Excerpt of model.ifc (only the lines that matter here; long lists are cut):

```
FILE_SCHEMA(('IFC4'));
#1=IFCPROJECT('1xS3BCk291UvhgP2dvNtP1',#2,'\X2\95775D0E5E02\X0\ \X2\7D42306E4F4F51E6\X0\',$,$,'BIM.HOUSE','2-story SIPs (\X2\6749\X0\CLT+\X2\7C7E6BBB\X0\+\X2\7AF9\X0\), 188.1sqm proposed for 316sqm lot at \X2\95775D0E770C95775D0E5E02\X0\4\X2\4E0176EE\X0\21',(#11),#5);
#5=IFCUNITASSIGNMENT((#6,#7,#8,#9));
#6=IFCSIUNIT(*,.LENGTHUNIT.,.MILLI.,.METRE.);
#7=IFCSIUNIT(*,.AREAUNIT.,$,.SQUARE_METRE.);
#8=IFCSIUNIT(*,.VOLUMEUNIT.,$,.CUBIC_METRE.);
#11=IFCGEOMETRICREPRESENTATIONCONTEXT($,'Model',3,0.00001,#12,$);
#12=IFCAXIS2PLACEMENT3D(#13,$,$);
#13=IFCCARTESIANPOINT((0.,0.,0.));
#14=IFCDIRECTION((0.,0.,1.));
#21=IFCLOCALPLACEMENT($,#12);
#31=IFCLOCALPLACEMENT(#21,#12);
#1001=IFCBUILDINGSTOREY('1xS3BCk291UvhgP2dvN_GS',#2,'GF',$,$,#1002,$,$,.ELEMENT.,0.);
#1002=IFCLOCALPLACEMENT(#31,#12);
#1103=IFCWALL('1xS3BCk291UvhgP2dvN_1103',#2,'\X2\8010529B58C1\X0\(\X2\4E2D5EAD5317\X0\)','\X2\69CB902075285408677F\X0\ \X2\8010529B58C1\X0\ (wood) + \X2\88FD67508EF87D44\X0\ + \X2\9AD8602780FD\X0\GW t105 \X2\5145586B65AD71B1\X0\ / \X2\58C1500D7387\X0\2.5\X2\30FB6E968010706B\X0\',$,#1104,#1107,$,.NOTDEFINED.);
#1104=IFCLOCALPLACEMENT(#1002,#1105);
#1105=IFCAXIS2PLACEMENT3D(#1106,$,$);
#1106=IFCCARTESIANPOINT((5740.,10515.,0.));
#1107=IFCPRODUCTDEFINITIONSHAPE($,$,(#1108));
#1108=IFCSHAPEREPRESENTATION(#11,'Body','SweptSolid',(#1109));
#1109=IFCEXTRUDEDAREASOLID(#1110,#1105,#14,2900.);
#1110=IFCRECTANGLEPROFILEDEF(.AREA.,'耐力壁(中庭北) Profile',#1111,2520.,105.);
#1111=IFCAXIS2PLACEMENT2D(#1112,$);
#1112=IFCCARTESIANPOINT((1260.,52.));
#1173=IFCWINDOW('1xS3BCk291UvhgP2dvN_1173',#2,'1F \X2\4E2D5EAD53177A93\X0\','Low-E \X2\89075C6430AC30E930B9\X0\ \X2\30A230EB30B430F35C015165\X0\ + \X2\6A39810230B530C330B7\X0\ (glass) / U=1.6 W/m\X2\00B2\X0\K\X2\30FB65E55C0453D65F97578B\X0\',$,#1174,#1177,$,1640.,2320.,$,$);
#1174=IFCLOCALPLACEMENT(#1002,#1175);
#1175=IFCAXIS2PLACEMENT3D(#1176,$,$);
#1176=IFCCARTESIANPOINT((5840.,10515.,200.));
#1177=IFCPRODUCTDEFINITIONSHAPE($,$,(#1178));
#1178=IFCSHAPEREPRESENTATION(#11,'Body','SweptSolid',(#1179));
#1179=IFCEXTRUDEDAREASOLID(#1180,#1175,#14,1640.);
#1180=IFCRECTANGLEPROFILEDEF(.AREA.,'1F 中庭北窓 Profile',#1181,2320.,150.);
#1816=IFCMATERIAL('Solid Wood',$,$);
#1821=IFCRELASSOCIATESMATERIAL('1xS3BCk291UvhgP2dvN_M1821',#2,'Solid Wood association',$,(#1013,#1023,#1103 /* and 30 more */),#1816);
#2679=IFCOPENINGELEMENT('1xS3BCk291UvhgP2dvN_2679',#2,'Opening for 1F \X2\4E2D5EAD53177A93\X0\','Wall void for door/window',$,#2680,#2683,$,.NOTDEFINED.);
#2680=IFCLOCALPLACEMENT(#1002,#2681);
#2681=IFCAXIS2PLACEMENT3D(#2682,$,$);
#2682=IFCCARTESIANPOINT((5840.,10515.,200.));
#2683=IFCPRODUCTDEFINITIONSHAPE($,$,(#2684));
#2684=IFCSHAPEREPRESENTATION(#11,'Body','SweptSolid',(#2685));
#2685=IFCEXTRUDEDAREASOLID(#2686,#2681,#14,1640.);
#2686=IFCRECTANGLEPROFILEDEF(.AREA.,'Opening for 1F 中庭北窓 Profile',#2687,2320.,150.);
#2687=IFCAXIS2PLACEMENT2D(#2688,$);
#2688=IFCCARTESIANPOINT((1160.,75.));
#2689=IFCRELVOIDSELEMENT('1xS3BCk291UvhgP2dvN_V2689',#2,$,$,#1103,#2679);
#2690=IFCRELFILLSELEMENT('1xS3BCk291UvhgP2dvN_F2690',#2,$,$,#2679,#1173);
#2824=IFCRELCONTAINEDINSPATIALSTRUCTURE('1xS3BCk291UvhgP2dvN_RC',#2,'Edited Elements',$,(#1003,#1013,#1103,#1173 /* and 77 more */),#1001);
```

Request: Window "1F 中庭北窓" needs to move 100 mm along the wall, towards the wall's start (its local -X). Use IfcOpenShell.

```python
import ifcopenshell
import ifcopenshell.api.geometry
import ifcopenshell.util.placement

model = ifcopenshell.open("model.ifc")

window = model.by_guid("1xS3BCk291UvhgP2dvN_1173")
opening = window.FillsVoids[0].RelatingOpeningElement
wall = opening.VoidsElements[0].RelatingBuildingElement

wall_matrix = ifcopenshell.util.placement.get_local_placement(wall.ObjectPlacement)
shift = wall_matrix[:3, 0] * -100.0
before = ifcopenshell.util.placement.get_local_placement(window.ObjectPlacement)[:3, 3].copy()

# The window is not placed relative to its opening, so move both.
for product in (opening, window):
    matrix = ifcopenshell.util.placement.get_local_placement(product.ObjectPlacement)
    matrix[:3, 3] += shift
    ifcopenshell.api.geometry.edit_object_placement(model, product=product, matrix=matrix, is_si=False)

after = ifcopenshell.util.placement.get_local_placement(window.ObjectPlacement)[:3, 3]
print("window moved by", (after - before).round(3) + 0.0)

model.write("model-out.ifc")
```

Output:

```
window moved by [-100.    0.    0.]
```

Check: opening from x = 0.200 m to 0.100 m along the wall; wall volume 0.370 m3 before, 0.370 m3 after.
